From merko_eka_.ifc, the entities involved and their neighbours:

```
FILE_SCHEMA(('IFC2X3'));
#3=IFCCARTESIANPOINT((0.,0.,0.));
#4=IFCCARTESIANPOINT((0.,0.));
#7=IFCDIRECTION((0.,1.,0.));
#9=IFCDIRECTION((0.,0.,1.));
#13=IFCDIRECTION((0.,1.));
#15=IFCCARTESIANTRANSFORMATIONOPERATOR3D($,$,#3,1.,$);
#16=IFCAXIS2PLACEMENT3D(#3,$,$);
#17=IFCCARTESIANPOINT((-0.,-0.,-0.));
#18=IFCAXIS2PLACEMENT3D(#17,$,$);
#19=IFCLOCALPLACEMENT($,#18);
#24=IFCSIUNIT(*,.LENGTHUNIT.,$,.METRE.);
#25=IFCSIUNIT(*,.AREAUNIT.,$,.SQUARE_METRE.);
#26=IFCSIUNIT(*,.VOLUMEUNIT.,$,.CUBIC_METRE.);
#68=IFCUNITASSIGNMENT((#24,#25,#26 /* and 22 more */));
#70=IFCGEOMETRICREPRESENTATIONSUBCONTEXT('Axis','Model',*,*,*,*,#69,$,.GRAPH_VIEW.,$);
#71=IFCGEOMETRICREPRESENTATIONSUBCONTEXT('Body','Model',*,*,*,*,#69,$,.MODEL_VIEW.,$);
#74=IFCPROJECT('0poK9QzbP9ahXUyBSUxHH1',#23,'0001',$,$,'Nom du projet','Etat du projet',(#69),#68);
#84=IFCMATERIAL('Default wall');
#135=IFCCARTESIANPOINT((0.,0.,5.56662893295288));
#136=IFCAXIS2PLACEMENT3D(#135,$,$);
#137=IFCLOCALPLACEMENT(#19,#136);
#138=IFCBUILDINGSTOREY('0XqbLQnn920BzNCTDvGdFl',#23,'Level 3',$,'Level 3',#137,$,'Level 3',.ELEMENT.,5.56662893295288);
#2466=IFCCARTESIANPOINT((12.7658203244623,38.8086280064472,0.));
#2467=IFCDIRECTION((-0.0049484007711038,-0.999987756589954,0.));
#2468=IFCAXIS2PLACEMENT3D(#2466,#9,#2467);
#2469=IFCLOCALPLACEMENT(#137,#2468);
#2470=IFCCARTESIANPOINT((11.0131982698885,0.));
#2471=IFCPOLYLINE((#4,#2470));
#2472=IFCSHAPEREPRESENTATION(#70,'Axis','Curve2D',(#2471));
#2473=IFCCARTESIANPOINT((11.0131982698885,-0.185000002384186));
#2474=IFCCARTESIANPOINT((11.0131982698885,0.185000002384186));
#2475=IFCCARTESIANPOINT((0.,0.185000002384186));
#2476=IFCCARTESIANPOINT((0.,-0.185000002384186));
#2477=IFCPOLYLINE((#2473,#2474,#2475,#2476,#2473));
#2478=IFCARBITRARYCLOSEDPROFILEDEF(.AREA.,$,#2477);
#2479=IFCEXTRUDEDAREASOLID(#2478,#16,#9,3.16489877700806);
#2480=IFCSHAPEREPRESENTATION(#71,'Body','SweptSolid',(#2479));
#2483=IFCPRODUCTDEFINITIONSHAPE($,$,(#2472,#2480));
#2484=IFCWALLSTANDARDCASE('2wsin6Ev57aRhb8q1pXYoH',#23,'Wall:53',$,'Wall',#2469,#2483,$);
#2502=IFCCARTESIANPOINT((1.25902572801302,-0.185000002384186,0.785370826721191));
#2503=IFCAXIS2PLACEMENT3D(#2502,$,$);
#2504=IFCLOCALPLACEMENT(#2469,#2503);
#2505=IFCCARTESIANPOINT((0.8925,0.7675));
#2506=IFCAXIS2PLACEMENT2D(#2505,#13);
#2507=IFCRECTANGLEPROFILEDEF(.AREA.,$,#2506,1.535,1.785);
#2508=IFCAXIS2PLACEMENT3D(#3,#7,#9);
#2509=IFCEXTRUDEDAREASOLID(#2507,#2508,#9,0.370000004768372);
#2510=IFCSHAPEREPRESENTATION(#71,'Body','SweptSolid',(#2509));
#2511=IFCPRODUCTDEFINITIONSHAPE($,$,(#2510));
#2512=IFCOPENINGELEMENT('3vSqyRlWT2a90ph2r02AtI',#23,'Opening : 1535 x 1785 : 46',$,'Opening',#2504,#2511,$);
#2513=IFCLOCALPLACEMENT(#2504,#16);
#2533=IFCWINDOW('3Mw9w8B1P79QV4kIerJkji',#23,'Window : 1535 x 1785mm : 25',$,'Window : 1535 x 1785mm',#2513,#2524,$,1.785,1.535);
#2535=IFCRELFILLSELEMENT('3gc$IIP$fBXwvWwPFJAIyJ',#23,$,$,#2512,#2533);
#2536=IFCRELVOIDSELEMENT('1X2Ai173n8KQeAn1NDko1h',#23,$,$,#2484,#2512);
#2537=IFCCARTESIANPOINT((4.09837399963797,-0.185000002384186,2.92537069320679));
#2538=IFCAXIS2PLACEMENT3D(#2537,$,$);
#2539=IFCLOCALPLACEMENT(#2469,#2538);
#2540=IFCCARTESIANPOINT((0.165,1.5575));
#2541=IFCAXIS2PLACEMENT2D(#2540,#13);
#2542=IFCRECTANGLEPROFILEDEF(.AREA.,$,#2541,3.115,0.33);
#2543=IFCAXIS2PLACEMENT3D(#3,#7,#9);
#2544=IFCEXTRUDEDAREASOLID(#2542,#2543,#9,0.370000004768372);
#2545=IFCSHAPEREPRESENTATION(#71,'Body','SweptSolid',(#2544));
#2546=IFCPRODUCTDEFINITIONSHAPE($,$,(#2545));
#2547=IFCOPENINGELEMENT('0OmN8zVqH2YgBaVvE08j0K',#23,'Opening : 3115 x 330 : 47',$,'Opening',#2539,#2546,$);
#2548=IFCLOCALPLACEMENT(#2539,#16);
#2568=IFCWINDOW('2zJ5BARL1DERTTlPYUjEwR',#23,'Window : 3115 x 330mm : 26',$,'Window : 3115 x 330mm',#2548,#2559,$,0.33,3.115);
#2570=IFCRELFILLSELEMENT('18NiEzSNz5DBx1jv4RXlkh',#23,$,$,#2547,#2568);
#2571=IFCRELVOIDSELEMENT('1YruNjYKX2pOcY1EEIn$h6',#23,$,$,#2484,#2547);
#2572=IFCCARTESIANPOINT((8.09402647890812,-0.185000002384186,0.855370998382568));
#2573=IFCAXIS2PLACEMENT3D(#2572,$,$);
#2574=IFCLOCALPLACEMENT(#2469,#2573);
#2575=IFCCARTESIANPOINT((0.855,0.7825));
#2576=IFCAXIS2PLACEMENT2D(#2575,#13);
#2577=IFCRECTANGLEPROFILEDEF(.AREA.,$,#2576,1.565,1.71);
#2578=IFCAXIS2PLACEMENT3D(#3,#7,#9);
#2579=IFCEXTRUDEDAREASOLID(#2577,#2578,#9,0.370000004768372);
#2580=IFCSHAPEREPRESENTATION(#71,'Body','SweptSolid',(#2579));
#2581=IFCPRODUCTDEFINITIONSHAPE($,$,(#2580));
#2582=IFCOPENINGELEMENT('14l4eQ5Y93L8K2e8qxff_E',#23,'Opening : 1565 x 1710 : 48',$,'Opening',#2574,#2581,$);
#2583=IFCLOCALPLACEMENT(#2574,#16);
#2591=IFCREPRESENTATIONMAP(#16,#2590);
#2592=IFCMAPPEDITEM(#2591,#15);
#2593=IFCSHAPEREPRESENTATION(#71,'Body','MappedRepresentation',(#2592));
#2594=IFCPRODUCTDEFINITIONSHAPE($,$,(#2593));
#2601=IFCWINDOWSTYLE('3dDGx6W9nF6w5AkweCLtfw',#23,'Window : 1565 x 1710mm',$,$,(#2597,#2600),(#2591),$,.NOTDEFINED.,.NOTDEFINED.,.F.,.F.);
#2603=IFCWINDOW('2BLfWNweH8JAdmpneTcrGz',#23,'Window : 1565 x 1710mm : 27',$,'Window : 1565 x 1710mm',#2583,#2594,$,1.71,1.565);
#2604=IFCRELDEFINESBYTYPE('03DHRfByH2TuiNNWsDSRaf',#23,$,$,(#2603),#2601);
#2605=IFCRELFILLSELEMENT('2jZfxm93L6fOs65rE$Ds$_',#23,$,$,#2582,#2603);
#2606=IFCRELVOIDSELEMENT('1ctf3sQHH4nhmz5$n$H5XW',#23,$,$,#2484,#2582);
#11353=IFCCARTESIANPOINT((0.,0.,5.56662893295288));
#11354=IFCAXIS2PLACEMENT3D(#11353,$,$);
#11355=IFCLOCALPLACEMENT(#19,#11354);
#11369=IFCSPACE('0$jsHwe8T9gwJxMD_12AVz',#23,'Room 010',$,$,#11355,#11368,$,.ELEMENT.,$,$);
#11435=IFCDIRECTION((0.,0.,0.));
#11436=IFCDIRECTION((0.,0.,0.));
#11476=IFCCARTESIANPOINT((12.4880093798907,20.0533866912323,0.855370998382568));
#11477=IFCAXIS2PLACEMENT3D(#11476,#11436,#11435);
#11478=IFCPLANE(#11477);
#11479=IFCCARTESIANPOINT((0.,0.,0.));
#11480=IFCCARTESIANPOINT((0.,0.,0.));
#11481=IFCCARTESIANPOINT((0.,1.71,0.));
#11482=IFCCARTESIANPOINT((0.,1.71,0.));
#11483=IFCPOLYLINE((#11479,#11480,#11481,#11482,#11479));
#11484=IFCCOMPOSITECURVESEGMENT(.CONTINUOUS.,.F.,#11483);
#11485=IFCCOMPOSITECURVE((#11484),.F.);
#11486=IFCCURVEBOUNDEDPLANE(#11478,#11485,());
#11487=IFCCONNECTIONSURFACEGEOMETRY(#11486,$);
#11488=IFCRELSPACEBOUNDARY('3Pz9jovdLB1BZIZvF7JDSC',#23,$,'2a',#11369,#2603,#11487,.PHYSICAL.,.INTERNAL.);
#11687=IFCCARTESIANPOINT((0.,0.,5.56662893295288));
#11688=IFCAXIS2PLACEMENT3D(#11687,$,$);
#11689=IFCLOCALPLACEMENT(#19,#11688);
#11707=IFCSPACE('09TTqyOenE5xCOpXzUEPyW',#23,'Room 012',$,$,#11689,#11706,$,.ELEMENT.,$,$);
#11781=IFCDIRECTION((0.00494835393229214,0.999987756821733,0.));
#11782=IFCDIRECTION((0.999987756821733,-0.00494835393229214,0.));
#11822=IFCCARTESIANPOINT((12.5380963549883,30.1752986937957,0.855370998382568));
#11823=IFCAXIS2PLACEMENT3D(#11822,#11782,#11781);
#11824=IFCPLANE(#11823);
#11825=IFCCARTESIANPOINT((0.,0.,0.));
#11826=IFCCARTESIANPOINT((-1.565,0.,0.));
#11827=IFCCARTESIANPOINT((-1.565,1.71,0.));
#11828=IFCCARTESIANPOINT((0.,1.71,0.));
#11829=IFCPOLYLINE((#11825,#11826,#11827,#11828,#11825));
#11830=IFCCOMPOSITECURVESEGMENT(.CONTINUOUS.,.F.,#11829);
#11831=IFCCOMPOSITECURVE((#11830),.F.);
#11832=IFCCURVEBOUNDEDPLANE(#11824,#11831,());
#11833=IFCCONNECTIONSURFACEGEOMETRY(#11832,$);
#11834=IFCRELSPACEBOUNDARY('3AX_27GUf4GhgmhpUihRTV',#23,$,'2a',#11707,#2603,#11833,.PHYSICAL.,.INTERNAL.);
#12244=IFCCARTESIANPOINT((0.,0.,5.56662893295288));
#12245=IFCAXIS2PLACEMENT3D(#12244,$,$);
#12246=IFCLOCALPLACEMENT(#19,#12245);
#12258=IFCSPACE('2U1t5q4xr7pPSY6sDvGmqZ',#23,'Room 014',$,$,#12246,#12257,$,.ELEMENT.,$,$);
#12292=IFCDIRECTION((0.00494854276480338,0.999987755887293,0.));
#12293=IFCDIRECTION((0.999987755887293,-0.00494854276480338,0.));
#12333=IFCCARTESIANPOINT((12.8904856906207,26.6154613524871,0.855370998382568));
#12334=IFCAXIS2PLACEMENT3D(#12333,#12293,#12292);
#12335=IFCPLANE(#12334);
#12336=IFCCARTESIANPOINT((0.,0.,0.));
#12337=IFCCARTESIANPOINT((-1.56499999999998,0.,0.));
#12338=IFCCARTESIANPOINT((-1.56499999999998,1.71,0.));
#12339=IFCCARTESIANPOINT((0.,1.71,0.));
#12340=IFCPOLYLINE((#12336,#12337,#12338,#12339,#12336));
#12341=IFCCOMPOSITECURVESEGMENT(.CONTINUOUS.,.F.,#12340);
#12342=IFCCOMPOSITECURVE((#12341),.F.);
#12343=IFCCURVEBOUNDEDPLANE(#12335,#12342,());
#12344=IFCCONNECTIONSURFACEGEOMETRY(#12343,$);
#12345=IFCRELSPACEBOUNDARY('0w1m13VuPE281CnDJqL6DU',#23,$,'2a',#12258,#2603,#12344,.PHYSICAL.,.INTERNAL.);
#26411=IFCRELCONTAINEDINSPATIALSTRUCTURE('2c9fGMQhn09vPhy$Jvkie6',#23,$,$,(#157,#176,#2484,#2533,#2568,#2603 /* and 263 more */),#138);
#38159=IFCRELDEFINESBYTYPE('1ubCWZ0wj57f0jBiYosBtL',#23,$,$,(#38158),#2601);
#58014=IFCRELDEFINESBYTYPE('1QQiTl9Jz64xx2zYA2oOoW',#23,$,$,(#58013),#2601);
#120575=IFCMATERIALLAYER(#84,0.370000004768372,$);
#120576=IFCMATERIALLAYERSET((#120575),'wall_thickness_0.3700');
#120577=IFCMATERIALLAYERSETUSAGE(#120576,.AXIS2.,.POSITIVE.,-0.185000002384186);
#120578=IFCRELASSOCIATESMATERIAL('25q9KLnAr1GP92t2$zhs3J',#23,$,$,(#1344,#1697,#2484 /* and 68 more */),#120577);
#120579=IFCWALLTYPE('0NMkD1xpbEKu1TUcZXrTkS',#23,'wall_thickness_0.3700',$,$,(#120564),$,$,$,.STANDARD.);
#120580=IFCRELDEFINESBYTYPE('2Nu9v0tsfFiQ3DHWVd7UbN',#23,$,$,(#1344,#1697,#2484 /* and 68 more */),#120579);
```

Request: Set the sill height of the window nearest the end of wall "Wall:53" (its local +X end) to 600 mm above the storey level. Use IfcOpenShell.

```python
import numpy as np
import ifcopenshell
import ifcopenshell.api.geometry
import ifcopenshell.geom
import ifcopenshell.util.element
import ifcopenshell.util.placement
import ifcopenshell.util.shape
import ifcopenshell.util.unit

model = ifcopenshell.open("merko_eka_.ifc")
unit_scale = ifcopenshell.util.unit.calculate_unit_scale(model)

window = model.by_guid("2BLfWNweH8JAdmpneTcrGz")
opening = window.FillsVoids[0].RelatingOpeningElement
storey = ifcopenshell.util.element.get_container(window, ifc_class="IfcBuildingStorey")
level = ifcopenshell.util.placement.get_local_placement(storey.ObjectPlacement)[2, 3]

# The opening's origin need not be at the sill, so measure its lowest point.
shape = ifcopenshell.geom.create_shape(ifcopenshell.geom.settings(), opening)
bottom = ifcopenshell.util.shape.get_shape_bottom_elevation(shape, shape.geometry) / unit_scale
dz = level + 0.6 - bottom

shift = np.array([0.0, 0.0, dz])
# The window is placed relative to its opening, so it follows when the opening moves.
matrix = ifcopenshell.util.placement.get_local_placement(opening.ObjectPlacement)
matrix[:3, 3] += shift
ifcopenshell.api.geometry.edit_object_placement(
    model, product=opening, matrix=matrix, is_si=False, should_transform_children=True
)

# Space boundary surfaces are stored in each space's coordinates; move them too.
for rel in window.ProvidesBoundaries:
    if not rel.ConnectionGeometry:
        continue
    surface = rel.ConnectionGeometry.SurfaceOnRelatingElement.BasisSurface
    space_matrix = ifcopenshell.util.placement.get_local_placement(rel.RelatingSpace.ObjectPlacement)
    point = np.array(surface.Position.Location.Coordinates) + space_matrix[:3, :3].T @ shift
    surface.Position = model.createIfcAxis2Placement3D(
        model.createIfcCartesianPoint(point.tolist()), surface.Position.Axis, surface.Position.RefDirection
    )

print(f"moved by {dz * unit_scale:+.3f} m")

model.write("merko_eka_-out.ifc")
```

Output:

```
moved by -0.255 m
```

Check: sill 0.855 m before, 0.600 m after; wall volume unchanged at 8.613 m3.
